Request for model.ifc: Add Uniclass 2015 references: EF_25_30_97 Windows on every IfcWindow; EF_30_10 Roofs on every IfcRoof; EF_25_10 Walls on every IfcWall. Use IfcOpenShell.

First a look at what the model holds.

```python
import ifcopenshell

model = ifcopenshell.open("model.ifc")
print(model.schema)
print("classifications:", [c.Name for c in model.by_type("IfcClassification")])
for ifc_class in ("IfcDoor", "IfcRoof", "IfcStair", "IfcWall", "IfcWindow"):
    print(ifc_class, len(model.by_type(ifc_class)))
```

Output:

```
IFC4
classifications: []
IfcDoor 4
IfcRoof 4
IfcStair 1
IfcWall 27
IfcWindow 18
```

```python
import ifcopenshell
import ifcopenshell.api.classification

model = ifcopenshell.open("model.ifc")

system = ifcopenshell.api.classification.add_classification(model, classification="Uniclass 2015")

codes = {
    "IfcWindow": ("EF_25_30_97", "Windows"),
    "IfcRoof": ("EF_30_10", "Roofs"),
    "IfcWall": ("EF_25_10", "Walls"),
}
for ifc_class, (code, name) in codes.items():
    products = model.by_type(ifc_class)
    ifcopenshell.api.classification.add_reference(
        model, products=products, classification=system, identification=code, name=name
    )
    print(code, len(products))

model.write("model_v2.ifc")
```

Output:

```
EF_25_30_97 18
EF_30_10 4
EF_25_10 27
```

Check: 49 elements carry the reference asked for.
